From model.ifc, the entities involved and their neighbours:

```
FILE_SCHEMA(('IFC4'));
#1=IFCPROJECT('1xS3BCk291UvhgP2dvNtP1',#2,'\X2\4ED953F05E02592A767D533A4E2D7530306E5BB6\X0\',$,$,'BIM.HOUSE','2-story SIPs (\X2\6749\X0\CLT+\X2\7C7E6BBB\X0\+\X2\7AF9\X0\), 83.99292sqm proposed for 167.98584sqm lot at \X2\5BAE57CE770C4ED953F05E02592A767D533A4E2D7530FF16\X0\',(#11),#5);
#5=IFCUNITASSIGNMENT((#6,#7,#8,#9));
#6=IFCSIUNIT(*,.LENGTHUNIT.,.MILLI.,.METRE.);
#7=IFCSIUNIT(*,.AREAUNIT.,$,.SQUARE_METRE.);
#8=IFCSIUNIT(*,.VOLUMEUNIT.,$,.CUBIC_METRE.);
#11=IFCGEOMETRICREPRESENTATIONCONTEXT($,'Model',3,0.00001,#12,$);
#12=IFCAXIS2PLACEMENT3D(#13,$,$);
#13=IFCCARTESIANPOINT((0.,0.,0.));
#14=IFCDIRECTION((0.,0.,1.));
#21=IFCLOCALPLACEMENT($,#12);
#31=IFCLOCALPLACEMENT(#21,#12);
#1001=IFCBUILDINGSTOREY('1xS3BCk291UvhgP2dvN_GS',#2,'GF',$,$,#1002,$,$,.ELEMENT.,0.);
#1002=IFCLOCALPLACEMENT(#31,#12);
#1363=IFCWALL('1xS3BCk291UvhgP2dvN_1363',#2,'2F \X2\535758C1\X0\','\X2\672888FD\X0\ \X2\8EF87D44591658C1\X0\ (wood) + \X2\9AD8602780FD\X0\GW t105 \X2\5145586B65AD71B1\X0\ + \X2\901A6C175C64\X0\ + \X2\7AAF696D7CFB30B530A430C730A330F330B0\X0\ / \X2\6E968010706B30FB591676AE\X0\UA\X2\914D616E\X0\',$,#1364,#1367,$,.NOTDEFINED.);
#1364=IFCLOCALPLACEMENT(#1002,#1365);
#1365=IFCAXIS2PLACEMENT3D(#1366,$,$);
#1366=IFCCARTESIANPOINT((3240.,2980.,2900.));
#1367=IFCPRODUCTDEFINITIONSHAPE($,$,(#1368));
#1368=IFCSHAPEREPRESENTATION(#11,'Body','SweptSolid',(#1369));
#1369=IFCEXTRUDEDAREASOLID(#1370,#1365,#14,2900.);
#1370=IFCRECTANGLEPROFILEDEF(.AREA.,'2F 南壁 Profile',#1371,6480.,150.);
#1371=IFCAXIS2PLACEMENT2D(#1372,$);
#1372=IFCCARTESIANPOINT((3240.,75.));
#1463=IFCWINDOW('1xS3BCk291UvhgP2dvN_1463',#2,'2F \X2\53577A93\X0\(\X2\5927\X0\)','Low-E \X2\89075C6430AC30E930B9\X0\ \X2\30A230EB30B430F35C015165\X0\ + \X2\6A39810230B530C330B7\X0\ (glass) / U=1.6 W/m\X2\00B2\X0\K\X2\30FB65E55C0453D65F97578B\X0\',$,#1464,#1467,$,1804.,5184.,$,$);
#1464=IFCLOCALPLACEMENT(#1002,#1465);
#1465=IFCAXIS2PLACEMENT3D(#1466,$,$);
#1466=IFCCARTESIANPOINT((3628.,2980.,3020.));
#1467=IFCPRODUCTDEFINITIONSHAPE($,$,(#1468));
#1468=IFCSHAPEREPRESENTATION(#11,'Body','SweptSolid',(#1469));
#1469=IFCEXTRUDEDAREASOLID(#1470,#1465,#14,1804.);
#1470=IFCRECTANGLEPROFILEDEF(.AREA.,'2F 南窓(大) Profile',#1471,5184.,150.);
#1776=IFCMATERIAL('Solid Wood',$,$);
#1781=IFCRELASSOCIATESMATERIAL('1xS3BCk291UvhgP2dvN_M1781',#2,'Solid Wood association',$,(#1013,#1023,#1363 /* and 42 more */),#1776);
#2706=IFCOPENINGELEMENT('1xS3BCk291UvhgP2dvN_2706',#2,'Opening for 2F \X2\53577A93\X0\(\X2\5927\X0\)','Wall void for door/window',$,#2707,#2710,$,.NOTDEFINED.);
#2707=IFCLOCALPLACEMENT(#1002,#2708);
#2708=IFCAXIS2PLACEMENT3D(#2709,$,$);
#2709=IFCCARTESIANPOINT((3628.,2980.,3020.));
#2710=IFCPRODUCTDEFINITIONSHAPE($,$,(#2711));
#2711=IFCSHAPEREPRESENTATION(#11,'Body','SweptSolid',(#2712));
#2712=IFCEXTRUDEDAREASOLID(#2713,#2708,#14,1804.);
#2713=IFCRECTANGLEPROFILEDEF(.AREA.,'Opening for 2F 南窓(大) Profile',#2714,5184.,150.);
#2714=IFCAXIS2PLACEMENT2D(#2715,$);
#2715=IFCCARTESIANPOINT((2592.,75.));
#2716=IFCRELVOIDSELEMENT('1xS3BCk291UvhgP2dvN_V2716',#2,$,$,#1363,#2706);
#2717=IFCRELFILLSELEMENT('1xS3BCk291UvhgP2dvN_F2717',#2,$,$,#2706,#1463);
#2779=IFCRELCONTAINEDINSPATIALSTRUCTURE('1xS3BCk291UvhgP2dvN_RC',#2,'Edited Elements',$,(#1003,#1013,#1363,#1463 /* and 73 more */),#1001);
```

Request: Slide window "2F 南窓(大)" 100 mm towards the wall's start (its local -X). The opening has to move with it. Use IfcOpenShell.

```python
import ifcopenshell
import ifcopenshell.api.geometry
import ifcopenshell.util.placement

model = ifcopenshell.open("model.ifc")

window = model.by_id(1463)
opening = window.FillsVoids[0].RelatingOpeningElement
wall = opening.VoidsElements[0].RelatingBuildingElement

wall_matrix = ifcopenshell.util.placement.get_local_placement(wall.ObjectPlacement)
shift = wall_matrix[:3, 0] * -100.0
before = ifcopenshell.util.placement.get_local_placement(window.ObjectPlacement)[:3, 3].copy()

# The window is not placed relative to its opening, so move both.
for product in (opening, window):
    matrix = ifcopenshell.util.placement.get_local_placement(product.ObjectPlacement)
    matrix[:3, 3] += shift
    ifcopenshell.api.geometry.edit_object_placement(model, product=product, matrix=matrix, is_si=False)

after = ifcopenshell.util.placement.get_local_placement(window.ObjectPlacement)[:3, 3]
print("window moved by", (after - before).round(3) + 0.0)

model.write("model_edited.ifc")
```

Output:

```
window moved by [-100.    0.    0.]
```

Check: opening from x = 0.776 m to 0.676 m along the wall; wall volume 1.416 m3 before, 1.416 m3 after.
